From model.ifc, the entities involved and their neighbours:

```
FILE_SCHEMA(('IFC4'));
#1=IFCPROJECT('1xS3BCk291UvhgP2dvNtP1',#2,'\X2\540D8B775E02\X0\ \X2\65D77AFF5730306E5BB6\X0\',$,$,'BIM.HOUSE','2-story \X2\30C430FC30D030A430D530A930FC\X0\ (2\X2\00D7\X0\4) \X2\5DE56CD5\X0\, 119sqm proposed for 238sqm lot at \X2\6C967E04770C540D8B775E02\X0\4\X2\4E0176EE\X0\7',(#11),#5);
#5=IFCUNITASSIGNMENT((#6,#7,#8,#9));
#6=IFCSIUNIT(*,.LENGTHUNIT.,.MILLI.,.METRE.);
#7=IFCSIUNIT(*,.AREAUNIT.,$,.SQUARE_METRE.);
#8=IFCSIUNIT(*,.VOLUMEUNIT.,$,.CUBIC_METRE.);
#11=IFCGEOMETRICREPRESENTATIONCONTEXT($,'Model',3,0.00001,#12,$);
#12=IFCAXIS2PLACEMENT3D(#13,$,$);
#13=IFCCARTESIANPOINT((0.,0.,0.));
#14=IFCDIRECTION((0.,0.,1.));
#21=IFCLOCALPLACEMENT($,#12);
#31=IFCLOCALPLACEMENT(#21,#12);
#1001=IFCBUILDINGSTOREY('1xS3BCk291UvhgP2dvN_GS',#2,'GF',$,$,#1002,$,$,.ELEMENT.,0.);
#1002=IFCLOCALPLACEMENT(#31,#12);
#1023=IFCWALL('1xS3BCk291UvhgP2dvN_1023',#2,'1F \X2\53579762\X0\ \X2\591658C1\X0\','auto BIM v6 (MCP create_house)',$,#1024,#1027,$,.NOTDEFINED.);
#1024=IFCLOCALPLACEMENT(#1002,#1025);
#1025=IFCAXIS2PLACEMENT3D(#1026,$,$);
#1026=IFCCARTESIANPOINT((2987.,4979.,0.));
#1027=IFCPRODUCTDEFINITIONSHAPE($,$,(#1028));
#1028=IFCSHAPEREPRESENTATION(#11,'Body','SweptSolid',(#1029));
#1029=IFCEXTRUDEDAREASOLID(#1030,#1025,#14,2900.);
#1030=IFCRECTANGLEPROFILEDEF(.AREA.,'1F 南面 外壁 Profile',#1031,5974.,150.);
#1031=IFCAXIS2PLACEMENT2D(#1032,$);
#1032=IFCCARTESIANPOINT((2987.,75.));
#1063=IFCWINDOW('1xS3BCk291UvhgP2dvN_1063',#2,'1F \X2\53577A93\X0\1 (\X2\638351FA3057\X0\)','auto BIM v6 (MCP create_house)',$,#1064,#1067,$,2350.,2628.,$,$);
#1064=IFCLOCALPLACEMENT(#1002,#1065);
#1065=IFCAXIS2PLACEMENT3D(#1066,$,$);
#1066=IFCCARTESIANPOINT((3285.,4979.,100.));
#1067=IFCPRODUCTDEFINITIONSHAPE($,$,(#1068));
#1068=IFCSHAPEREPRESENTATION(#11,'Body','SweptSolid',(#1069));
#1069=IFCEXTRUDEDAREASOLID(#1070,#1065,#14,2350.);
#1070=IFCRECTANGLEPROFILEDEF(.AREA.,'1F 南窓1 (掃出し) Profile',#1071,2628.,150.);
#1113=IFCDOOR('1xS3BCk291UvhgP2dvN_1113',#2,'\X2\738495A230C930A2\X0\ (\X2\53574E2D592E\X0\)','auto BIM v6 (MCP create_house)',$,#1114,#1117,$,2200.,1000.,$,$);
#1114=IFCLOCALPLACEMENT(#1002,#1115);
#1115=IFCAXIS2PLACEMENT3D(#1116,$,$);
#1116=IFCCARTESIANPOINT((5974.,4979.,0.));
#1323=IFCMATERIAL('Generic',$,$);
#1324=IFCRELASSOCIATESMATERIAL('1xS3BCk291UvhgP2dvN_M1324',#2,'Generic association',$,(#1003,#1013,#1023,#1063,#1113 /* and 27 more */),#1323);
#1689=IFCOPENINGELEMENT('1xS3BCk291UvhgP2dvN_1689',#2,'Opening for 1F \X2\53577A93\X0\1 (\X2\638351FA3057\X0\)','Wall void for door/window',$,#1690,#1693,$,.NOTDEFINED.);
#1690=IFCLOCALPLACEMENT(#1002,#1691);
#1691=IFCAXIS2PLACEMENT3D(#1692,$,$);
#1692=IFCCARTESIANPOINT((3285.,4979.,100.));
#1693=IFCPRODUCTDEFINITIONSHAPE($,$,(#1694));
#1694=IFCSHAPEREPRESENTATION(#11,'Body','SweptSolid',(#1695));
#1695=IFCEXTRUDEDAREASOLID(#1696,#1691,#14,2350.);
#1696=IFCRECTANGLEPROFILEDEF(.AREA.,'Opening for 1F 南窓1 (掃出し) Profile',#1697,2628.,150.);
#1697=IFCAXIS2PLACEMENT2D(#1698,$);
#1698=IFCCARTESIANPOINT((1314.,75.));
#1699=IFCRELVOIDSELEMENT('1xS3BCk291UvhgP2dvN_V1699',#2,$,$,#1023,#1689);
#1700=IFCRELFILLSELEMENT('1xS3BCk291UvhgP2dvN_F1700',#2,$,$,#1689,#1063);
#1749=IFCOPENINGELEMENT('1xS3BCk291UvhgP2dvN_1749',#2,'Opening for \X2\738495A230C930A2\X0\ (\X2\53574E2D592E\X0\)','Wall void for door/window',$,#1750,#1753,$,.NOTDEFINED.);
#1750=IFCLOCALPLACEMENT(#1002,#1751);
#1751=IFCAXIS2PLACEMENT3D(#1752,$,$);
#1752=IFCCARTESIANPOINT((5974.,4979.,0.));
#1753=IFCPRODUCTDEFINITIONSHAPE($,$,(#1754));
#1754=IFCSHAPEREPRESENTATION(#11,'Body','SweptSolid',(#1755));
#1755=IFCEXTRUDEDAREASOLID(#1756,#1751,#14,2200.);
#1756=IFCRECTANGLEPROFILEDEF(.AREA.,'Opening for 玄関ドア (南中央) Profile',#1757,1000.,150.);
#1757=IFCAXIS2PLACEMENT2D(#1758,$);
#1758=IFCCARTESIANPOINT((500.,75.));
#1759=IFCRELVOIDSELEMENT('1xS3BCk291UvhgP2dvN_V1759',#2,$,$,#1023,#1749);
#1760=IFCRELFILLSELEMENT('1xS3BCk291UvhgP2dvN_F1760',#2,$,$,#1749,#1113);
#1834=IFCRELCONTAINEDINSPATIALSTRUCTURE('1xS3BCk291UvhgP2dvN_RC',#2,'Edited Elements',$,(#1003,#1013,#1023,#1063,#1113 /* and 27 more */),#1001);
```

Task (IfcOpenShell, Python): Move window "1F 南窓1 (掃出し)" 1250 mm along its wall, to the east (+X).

```python
import ifcopenshell
import ifcopenshell.api.geometry
import ifcopenshell.util.placement
import ifcopenshell.util.unit

model = ifcopenshell.open("model.ifc")
unit_scale = ifcopenshell.util.unit.calculate_unit_scale(model)

window = model.by_guid("1xS3BCk291UvhgP2dvN_1063")
opening = window.FillsVoids[0].RelatingOpeningElement
wall = opening.VoidsElements[0].RelatingBuildingElement

wall_matrix = ifcopenshell.util.placement.get_local_placement(wall.ObjectPlacement)
shift = wall_matrix[:3, 0] * 1.25 / unit_scale
before = ifcopenshell.util.placement.get_local_placement(window.ObjectPlacement)[:3, 3].copy()

# The window is not placed relative to its opening, so move both.
for product in (opening, window):
    matrix = ifcopenshell.util.placement.get_local_placement(product.ObjectPlacement)
    matrix[:3, 3] += shift
    ifcopenshell.api.geometry.edit_object_placement(model, product=product, matrix=matrix, is_si=False)

after = ifcopenshell.util.placement.get_local_placement(window.ObjectPlacement)[:3, 3]
print("window moved by", (after - before).round(3) + 0.0)

model.write("model_v2.ifc")
```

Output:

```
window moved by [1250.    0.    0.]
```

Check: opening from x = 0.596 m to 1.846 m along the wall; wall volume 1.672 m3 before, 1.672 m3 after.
